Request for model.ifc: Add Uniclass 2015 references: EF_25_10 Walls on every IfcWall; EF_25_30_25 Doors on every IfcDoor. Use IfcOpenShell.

First a look at what the model holds.

```python
import ifcopenshell

model = ifcopenshell.open("model.ifc")
print(model.schema)
print("classifications:", [c.Name for c in model.by_type("IfcClassification")])
for ifc_class in ("IfcDoor", "IfcRoof", "IfcStair", "IfcWall", "IfcWindow"):
    print(ifc_class, len(model.by_type(ifc_class)))
```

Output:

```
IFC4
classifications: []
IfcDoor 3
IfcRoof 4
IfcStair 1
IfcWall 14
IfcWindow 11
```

```python
import ifcopenshell
import ifcopenshell.api.classification

model = ifcopenshell.open("model.ifc")

system = ifcopenshell.api.classification.add_classification(model, classification="Uniclass 2015")

codes = {
    "IfcWall": ("EF_25_10", "Walls"),
    "IfcDoor": ("EF_25_30_25", "Doors"),
}
for ifc_class, (code, name) in codes.items():
    products = model.by_type(ifc_class)
    ifcopenshell.api.classification.add_reference(
        model, products=products, classification=system, identification=code, name=name
    )
    print(code, len(products))

model.write("model_edited.ifc")
```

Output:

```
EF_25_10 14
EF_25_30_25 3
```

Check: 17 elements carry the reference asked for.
